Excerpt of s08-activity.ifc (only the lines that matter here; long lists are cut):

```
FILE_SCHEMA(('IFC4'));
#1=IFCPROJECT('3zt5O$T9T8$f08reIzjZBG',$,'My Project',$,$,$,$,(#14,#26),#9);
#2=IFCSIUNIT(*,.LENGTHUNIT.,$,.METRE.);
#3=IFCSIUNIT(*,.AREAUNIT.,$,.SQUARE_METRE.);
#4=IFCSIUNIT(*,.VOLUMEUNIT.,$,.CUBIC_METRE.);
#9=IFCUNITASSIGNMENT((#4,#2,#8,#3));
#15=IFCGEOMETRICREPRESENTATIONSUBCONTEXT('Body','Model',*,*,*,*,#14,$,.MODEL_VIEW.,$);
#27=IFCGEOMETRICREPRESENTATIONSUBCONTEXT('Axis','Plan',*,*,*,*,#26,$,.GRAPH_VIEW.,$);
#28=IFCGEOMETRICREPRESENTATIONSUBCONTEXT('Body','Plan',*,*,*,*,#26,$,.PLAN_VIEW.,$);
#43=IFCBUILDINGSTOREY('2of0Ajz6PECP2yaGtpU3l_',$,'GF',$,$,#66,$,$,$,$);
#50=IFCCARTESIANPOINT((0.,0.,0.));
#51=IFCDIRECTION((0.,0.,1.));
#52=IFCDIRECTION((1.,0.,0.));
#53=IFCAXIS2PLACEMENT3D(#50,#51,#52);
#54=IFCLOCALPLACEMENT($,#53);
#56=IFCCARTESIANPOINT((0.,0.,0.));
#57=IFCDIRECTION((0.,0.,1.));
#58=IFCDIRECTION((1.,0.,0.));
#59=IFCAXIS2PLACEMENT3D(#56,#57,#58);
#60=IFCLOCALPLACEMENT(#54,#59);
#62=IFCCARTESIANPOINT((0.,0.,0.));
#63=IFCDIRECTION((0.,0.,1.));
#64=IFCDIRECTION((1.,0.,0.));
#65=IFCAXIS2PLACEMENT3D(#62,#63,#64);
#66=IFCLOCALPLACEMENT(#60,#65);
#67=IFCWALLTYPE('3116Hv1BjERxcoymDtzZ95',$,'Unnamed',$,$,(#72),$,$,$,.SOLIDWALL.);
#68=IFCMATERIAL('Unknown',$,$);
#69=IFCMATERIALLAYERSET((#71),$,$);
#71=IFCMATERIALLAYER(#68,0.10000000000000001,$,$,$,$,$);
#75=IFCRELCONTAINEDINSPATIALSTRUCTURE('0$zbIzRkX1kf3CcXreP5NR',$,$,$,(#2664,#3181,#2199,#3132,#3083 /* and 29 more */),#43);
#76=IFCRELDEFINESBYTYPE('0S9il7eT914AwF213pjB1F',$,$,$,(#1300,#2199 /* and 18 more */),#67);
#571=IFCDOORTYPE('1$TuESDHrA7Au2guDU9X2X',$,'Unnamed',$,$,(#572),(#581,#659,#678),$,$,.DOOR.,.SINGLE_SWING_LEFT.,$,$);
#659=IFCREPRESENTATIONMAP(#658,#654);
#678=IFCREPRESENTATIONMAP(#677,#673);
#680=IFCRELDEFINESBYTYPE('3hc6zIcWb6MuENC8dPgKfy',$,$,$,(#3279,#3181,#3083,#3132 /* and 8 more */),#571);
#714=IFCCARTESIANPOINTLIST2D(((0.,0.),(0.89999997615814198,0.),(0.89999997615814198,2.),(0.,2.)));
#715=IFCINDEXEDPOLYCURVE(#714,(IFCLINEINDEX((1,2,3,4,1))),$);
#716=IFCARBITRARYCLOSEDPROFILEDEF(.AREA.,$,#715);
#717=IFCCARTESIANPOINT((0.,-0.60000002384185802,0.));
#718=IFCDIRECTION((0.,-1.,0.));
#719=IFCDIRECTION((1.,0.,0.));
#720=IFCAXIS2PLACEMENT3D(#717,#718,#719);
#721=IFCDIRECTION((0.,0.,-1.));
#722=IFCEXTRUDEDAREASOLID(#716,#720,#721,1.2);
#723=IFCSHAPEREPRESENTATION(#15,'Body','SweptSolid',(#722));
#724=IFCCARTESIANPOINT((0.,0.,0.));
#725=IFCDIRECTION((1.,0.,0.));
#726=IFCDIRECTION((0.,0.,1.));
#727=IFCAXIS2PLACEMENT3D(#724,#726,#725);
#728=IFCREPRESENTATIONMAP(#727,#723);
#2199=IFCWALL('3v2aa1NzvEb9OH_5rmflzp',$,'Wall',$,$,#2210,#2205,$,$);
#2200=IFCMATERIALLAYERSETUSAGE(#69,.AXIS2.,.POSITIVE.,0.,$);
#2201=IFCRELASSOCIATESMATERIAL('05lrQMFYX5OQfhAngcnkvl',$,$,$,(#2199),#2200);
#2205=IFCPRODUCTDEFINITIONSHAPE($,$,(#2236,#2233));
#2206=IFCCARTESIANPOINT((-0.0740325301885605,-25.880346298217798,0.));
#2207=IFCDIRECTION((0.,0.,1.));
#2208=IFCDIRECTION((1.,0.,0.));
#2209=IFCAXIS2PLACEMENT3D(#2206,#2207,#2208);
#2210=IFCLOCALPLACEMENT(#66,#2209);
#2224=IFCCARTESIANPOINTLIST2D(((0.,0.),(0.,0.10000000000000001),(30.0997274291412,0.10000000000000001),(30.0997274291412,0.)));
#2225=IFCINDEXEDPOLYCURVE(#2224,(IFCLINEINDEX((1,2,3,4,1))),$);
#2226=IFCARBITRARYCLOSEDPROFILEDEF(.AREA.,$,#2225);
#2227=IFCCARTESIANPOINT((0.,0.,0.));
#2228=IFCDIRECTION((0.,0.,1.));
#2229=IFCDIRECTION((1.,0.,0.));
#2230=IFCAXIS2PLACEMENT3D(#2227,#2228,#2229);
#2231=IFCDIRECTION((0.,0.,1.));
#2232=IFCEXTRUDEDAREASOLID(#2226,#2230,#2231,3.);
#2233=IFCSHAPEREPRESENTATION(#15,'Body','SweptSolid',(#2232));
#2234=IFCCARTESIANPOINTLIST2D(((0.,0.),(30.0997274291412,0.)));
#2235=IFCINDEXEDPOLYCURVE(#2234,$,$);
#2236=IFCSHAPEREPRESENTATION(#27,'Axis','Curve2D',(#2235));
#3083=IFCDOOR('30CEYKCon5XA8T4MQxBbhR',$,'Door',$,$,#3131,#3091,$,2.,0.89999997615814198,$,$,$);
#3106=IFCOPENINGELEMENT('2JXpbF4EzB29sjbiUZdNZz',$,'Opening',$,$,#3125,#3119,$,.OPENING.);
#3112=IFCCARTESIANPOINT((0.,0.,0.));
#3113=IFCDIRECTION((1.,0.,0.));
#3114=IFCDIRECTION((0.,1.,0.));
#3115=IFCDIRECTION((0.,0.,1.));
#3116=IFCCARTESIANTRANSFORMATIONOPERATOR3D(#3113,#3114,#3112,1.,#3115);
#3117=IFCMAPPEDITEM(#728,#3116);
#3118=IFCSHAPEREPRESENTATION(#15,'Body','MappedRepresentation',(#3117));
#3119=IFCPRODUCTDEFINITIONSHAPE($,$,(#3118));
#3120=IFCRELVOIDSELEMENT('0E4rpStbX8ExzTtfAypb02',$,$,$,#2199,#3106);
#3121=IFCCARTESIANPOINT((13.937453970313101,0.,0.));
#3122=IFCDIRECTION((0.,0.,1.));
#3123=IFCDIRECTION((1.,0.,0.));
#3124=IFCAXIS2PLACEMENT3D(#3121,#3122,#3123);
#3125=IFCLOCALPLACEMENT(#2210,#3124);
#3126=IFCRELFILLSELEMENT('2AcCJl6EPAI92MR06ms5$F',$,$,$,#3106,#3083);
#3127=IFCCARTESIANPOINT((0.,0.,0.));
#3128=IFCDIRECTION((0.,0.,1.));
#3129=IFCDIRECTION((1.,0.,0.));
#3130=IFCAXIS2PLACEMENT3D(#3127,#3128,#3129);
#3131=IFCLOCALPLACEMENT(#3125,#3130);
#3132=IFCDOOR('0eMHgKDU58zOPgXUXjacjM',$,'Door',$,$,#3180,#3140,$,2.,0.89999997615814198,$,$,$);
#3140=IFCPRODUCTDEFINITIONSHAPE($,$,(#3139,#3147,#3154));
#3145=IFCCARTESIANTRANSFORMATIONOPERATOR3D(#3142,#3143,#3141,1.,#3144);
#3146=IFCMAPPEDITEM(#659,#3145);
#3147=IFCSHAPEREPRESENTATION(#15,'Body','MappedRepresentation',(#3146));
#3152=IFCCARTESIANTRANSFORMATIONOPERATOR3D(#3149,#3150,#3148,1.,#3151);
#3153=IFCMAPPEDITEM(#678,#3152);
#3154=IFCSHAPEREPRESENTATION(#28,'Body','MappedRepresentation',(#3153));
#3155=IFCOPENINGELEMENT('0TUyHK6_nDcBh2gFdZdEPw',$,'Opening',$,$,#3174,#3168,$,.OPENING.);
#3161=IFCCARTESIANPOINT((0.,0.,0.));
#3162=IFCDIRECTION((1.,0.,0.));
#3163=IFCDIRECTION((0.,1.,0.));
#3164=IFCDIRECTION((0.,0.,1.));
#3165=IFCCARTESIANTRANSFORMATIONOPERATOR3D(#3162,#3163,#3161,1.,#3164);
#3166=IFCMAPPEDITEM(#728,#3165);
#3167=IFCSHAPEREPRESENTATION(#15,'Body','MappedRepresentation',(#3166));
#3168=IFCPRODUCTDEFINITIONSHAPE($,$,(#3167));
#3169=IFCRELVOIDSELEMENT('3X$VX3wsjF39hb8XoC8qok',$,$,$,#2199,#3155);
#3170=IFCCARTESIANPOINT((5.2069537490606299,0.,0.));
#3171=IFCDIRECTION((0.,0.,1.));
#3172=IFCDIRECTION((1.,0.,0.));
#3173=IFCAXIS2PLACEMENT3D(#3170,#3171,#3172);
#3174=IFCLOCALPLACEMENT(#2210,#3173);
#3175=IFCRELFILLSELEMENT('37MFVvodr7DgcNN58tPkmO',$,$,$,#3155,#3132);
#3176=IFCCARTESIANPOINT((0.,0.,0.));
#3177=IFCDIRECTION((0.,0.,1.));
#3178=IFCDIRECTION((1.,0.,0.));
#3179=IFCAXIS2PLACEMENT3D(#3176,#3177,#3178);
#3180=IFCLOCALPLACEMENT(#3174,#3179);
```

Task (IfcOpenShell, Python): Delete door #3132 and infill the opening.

```python
import ifcopenshell
import ifcopenshell.api.feature
import ifcopenshell.api.root
import ifcopenshell.geom
import ifcopenshell.util.shape

model = ifcopenshell.open("s08-activity.ifc")
settings = ifcopenshell.geom.settings()


def volume(element):
    """Net volume in cubic metres, openings subtracted."""
    shape = ifcopenshell.geom.create_shape(settings, element)
    return ifcopenshell.util.shape.get_volume(shape.geometry)


door = model.by_guid("0eMHgKDU58zOPgXUXjacjM")
opening = door.FillsVoids[0].RelatingOpeningElement
wall = opening.VoidsElements[0].RelatingBuildingElement
before = volume(wall)

ifcopenshell.api.root.remove_product(model, product=door)
ifcopenshell.api.feature.remove_feature(model, feature=opening)

after = volume(wall)

print(f"wall volume {before:.3f} -> {after:.3f} m3")

model.write("s08-activity_v2.ifc")
```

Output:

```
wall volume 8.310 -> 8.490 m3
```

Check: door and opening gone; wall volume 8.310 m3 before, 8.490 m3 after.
